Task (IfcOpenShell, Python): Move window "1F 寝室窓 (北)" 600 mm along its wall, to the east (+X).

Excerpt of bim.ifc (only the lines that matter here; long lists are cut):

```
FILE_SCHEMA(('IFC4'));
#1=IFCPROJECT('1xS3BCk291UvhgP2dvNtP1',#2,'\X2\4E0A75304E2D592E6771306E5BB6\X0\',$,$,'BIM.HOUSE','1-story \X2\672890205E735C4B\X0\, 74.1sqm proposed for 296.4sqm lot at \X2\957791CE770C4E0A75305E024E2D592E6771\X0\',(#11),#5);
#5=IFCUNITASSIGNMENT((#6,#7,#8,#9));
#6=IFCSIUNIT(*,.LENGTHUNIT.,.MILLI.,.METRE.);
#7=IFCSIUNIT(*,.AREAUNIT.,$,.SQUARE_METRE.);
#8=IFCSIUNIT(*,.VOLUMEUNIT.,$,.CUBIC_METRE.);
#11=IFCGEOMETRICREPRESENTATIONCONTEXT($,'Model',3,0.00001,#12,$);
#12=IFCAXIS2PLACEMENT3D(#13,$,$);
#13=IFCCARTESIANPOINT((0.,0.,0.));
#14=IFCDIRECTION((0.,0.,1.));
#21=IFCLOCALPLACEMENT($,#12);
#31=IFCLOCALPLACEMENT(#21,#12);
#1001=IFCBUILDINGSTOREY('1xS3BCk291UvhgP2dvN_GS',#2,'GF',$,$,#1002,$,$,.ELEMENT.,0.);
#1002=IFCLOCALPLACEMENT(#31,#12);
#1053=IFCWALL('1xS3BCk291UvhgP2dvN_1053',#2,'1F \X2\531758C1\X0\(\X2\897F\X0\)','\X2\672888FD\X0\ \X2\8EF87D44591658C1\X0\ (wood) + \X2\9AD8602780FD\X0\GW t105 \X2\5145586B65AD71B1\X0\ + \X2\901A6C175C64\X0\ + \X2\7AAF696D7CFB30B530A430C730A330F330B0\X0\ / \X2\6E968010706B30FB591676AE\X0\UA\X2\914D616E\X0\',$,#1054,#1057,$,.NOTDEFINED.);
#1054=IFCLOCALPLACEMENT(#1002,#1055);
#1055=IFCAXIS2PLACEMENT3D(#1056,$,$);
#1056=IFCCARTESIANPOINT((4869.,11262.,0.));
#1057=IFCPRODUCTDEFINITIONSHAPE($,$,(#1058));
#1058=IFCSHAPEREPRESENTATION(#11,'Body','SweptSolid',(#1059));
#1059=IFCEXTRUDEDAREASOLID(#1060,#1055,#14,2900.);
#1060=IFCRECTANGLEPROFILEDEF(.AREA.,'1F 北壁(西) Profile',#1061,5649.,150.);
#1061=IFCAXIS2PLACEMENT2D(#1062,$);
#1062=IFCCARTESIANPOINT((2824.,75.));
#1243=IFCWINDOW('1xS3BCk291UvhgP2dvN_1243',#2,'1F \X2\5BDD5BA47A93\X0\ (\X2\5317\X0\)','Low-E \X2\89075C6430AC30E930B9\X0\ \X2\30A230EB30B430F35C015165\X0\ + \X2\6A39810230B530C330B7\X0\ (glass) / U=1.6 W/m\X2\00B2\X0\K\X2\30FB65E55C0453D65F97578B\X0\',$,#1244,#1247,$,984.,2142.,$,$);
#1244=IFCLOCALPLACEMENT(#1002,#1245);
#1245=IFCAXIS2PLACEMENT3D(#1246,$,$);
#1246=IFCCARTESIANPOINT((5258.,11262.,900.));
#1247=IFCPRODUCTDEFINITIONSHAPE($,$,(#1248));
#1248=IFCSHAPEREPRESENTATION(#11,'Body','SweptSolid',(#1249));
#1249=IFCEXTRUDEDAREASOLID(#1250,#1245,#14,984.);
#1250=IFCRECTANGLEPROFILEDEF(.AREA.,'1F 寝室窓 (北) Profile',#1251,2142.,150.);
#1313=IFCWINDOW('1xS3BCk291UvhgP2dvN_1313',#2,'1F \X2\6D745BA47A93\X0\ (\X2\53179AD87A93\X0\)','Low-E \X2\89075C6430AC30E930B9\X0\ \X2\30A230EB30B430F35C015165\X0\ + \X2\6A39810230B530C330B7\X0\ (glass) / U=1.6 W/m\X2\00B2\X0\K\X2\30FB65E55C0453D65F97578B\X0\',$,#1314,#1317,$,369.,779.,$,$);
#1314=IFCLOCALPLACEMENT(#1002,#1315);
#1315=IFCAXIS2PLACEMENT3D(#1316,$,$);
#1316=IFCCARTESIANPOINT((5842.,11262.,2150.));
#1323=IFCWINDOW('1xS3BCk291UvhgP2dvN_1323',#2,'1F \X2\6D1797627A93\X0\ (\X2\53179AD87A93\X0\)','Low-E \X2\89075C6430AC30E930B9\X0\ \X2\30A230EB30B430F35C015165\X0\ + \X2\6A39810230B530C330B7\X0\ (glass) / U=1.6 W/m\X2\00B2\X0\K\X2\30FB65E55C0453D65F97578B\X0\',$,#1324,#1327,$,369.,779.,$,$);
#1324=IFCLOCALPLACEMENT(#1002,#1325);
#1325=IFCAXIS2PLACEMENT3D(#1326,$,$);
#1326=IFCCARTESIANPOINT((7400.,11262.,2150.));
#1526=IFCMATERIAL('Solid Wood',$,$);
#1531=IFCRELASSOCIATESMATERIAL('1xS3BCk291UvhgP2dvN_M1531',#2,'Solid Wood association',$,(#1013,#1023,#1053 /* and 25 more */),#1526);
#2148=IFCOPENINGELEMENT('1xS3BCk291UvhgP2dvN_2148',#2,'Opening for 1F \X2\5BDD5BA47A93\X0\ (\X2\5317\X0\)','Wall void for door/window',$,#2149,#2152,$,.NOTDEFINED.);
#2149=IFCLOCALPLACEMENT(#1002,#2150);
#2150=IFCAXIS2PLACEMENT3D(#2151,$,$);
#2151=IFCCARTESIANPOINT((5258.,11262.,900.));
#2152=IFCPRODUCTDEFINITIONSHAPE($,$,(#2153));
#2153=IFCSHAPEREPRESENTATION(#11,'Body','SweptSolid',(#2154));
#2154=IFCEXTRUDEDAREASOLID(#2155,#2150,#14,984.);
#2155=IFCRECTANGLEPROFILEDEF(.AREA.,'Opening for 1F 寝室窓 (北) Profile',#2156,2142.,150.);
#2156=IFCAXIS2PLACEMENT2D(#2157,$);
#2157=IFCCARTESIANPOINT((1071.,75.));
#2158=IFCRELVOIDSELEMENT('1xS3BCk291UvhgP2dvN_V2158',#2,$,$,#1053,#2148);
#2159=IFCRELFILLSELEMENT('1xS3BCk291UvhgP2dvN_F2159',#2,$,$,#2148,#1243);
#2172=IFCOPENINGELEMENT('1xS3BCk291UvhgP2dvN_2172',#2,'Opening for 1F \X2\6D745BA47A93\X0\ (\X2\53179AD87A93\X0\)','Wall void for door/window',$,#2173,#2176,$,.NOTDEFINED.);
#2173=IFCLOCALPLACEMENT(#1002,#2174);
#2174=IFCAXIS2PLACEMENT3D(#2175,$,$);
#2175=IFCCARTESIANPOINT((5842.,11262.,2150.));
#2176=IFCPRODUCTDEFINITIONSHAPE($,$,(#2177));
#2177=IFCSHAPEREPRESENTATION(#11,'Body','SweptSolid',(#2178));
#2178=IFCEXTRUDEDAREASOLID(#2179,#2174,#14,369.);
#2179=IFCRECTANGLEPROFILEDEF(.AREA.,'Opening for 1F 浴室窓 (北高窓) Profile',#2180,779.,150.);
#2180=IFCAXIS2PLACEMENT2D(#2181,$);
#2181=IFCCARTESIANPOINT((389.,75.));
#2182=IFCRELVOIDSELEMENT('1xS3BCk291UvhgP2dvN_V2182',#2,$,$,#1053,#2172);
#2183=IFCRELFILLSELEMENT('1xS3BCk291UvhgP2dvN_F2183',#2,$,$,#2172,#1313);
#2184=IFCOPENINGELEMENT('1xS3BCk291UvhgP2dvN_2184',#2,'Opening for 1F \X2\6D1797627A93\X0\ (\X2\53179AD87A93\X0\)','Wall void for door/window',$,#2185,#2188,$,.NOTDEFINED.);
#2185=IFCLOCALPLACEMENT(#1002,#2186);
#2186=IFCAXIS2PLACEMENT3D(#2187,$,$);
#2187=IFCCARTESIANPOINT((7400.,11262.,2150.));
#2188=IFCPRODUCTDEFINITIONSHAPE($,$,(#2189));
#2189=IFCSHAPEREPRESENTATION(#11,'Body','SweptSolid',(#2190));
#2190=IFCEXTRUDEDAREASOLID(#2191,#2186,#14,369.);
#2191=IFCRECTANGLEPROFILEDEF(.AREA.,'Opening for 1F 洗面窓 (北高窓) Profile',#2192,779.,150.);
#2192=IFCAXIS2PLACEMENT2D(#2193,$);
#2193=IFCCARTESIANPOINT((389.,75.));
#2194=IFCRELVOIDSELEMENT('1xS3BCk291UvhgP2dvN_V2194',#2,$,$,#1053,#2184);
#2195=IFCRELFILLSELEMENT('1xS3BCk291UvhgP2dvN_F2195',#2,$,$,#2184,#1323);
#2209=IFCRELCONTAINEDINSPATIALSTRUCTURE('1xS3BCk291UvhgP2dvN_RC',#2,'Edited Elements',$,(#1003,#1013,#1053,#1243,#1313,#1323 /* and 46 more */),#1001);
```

```python
import ifcopenshell
import ifcopenshell.api.geometry
import ifcopenshell.util.placement
import ifcopenshell.util.unit

model = ifcopenshell.open("bim.ifc")
unit_scale = ifcopenshell.util.unit.calculate_unit_scale(model)

window = model.by_guid("1xS3BCk291UvhgP2dvN_1243")
opening = window.FillsVoids[0].RelatingOpeningElement
wall = opening.VoidsElements[0].RelatingBuildingElement

wall_matrix = ifcopenshell.util.placement.get_local_placement(wall.ObjectPlacement)
shift = wall_matrix[:3, 0] * 0.6 / unit_scale
before = ifcopenshell.util.placement.get_local_placement(window.ObjectPlacement)[:3, 3].copy()

# The window is not placed relative to its opening, so move both.
for product in (opening, window):
    matrix = ifcopenshell.util.placement.get_local_placement(product.ObjectPlacement)
    matrix[:3, 3] += shift
    ifcopenshell.api.geometry.edit_object_placement(model, product=product, matrix=matrix, is_si=False)

after = ifcopenshell.util.placement.get_local_placement(window.ObjectPlacement)[:3, 3]
print("window moved by", (after - before).round(3) + 0.0)

model.write("bim-out.ifc")
```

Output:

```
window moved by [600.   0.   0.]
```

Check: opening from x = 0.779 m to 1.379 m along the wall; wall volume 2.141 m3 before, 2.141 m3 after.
